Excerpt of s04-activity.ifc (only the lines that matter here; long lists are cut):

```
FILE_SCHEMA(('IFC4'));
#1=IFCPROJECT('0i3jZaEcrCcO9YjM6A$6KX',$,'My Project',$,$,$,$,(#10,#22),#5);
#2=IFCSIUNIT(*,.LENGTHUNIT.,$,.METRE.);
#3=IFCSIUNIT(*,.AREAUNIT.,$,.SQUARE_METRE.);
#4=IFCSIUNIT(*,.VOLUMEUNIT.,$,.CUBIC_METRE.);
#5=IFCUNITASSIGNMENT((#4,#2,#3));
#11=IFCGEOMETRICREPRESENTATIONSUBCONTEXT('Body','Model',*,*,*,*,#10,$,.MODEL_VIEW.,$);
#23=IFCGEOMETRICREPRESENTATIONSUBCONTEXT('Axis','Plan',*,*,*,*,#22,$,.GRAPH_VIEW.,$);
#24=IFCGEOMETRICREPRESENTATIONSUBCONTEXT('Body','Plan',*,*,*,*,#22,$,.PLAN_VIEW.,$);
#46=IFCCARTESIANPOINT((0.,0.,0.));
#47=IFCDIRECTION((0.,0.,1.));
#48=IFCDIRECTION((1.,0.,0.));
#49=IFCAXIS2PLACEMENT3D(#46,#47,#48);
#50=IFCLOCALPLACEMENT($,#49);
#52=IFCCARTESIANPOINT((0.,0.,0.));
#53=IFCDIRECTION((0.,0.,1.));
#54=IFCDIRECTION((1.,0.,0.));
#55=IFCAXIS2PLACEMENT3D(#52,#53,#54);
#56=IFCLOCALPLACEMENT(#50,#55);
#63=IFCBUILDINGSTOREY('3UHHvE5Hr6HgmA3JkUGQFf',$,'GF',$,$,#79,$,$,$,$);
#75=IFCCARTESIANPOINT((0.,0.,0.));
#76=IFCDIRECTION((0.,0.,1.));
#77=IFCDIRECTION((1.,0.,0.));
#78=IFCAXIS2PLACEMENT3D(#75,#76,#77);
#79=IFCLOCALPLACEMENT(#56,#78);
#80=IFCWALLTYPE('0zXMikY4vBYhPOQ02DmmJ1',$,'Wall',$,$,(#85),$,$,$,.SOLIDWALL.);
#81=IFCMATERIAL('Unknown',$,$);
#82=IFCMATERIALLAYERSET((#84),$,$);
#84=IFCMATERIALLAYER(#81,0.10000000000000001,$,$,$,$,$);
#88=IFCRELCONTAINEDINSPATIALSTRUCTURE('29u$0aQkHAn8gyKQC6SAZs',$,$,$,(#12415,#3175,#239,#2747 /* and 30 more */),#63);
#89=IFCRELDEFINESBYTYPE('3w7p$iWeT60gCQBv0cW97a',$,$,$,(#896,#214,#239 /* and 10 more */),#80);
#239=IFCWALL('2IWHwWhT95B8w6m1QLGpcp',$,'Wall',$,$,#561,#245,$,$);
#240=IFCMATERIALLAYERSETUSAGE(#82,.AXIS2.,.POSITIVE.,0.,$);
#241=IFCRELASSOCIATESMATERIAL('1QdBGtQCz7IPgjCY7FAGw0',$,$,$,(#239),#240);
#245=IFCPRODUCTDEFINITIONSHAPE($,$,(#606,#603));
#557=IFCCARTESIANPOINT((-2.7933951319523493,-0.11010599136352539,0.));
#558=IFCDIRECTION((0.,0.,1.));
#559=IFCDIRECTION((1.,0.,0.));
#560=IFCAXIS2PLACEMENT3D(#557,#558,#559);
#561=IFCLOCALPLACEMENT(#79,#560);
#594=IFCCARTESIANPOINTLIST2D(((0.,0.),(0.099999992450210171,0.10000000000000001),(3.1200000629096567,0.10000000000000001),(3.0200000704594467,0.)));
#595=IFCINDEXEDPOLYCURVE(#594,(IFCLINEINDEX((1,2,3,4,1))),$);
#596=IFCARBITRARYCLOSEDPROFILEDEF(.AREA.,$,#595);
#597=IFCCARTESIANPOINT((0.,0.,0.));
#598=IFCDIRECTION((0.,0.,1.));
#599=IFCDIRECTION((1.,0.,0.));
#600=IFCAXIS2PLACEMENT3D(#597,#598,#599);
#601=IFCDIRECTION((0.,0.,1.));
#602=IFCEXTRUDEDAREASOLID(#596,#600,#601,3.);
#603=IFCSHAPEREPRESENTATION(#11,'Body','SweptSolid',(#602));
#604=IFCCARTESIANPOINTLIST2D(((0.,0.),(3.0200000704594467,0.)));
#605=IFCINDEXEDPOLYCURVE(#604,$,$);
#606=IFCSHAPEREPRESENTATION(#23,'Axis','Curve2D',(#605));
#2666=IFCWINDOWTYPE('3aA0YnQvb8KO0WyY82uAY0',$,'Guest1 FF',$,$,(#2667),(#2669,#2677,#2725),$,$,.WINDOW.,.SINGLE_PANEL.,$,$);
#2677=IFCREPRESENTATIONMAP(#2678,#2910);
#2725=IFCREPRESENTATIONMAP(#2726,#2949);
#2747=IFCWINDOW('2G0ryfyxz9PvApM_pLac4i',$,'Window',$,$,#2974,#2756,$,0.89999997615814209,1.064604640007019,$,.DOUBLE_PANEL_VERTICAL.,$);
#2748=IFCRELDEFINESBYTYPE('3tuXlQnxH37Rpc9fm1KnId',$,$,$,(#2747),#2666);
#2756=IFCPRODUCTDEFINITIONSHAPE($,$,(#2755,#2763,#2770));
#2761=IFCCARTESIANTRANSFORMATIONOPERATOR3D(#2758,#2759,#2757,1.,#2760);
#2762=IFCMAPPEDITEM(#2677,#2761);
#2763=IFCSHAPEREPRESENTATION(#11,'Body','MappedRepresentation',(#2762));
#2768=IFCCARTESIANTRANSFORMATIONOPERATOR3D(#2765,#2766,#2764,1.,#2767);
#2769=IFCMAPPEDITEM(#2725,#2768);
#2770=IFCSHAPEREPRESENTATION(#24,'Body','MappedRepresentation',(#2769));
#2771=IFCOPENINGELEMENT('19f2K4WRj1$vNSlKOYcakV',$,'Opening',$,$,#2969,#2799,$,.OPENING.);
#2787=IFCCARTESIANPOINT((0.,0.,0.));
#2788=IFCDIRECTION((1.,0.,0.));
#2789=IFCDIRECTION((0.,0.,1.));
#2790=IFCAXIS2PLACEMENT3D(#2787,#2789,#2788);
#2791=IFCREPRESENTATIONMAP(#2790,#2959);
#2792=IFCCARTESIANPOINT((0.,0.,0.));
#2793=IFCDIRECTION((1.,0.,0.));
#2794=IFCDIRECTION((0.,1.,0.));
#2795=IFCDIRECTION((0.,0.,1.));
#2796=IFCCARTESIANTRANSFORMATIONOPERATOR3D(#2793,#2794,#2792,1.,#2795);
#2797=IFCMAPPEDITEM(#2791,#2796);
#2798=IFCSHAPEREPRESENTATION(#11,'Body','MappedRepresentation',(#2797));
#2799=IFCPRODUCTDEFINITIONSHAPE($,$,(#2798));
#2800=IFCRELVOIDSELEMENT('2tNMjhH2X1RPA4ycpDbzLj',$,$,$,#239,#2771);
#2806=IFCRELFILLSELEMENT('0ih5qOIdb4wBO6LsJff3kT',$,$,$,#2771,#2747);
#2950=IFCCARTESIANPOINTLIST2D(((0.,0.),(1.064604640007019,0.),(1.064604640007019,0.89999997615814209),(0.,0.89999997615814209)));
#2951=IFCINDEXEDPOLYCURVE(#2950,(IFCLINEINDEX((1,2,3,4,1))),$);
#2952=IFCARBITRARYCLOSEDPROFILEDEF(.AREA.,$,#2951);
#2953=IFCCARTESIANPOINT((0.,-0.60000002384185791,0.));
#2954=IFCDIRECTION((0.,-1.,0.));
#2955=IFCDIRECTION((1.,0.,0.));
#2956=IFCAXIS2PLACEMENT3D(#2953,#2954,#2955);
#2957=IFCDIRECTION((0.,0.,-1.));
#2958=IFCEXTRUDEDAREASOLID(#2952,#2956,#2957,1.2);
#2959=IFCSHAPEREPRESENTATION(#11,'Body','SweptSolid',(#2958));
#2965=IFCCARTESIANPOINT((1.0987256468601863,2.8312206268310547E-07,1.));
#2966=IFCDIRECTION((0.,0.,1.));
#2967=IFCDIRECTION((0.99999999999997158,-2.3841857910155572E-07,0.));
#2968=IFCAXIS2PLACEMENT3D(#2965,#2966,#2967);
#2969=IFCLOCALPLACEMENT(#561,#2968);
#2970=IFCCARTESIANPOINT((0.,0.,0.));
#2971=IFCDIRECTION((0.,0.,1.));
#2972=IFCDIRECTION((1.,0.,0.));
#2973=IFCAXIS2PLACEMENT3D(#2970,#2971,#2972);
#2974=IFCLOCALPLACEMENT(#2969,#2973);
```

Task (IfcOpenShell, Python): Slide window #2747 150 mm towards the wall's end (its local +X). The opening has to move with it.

```python
import ifcopenshell
import ifcopenshell.api.geometry
import ifcopenshell.util.placement

model = ifcopenshell.open("s04-activity.ifc")

window = model.by_guid("2G0ryfyxz9PvApM_pLac4i")
opening = window.FillsVoids[0].RelatingOpeningElement
wall = opening.VoidsElements[0].RelatingBuildingElement

wall_matrix = ifcopenshell.util.placement.get_local_placement(wall.ObjectPlacement)
shift = wall_matrix[:3, 0] * 0.15
before = ifcopenshell.util.placement.get_local_placement(window.ObjectPlacement)[:3, 3].copy()

# The window is placed relative to its opening, so it follows when the opening moves.
matrix = ifcopenshell.util.placement.get_local_placement(opening.ObjectPlacement)
matrix[:3, 3] += shift
ifcopenshell.api.geometry.edit_object_placement(
    model, product=opening, matrix=matrix, is_si=False, should_transform_children=True
)

after = ifcopenshell.util.placement.get_local_placement(window.ObjectPlacement)[:3, 3]
print("window moved by", (after - before).round(3) + 0.0)

model.write("s04-activity_updated.ifc")
```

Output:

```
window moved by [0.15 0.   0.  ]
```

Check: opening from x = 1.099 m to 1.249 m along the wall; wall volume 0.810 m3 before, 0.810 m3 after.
